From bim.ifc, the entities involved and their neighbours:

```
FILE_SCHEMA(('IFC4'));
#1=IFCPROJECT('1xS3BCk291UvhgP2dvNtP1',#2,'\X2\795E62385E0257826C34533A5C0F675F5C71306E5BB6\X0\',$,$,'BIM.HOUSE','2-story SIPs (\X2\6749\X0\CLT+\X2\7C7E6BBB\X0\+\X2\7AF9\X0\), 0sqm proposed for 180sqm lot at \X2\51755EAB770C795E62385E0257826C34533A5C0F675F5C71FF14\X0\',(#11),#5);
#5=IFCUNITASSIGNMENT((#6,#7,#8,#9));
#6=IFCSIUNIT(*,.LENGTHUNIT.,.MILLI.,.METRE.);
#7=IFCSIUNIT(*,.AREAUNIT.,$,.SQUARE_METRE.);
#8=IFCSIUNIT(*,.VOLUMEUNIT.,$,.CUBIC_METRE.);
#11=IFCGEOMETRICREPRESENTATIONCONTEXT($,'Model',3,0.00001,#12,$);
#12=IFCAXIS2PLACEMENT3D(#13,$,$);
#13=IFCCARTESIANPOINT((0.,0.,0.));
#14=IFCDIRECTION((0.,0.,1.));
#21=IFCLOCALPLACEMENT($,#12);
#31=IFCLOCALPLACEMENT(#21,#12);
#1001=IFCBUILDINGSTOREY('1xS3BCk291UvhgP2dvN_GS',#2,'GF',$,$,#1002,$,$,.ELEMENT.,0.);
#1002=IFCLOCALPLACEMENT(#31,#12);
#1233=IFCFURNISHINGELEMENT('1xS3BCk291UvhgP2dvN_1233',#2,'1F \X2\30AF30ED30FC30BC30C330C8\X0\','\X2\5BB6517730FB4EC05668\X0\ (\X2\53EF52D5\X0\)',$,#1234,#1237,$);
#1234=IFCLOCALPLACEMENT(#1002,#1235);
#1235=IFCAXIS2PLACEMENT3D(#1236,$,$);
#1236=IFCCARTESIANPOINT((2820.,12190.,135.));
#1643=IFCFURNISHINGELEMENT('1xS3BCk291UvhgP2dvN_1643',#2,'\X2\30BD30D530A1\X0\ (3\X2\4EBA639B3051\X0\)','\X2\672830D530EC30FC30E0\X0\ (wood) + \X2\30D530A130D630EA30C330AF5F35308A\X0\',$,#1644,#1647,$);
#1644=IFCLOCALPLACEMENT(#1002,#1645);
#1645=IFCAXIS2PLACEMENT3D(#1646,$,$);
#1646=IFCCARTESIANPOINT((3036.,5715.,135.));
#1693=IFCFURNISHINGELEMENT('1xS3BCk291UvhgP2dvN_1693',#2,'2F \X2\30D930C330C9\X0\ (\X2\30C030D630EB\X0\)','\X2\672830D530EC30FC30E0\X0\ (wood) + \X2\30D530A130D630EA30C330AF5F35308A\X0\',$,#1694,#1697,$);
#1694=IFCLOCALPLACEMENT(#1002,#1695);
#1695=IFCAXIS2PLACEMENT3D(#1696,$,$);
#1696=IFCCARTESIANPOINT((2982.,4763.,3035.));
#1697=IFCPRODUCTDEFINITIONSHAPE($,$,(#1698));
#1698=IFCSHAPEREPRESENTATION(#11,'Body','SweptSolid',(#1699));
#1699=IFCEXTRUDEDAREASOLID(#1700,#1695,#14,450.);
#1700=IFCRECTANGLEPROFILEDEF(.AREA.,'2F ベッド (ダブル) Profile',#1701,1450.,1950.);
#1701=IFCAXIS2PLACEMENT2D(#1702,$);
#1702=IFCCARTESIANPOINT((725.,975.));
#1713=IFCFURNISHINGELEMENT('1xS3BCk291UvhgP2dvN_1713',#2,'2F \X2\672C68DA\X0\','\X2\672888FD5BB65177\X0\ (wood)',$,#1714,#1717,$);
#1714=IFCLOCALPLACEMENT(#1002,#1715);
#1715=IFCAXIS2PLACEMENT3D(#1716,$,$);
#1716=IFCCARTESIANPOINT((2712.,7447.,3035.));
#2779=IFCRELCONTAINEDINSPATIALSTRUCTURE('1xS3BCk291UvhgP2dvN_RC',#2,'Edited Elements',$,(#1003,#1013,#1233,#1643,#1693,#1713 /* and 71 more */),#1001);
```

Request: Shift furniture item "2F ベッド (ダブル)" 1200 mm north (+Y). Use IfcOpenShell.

```python
import ifcopenshell
import ifcopenshell.api.geometry
import ifcopenshell.util.placement

model = ifcopenshell.open("bim.ifc")

item = model.by_id(1693)
matrix = ifcopenshell.util.placement.get_local_placement(item.ObjectPlacement)
matrix[1, 3] += 1200.0
ifcopenshell.api.geometry.edit_object_placement(model, product=item, matrix=matrix, is_si=False)

print(ifcopenshell.util.placement.get_local_placement(item.ObjectPlacement).round(3) + 0.0)

model.write("bim_v2.ifc")
```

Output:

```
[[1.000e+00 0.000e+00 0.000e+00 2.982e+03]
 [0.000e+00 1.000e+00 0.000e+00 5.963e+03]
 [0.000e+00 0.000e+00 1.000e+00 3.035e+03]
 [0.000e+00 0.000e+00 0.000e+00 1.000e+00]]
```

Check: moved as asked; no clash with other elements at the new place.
